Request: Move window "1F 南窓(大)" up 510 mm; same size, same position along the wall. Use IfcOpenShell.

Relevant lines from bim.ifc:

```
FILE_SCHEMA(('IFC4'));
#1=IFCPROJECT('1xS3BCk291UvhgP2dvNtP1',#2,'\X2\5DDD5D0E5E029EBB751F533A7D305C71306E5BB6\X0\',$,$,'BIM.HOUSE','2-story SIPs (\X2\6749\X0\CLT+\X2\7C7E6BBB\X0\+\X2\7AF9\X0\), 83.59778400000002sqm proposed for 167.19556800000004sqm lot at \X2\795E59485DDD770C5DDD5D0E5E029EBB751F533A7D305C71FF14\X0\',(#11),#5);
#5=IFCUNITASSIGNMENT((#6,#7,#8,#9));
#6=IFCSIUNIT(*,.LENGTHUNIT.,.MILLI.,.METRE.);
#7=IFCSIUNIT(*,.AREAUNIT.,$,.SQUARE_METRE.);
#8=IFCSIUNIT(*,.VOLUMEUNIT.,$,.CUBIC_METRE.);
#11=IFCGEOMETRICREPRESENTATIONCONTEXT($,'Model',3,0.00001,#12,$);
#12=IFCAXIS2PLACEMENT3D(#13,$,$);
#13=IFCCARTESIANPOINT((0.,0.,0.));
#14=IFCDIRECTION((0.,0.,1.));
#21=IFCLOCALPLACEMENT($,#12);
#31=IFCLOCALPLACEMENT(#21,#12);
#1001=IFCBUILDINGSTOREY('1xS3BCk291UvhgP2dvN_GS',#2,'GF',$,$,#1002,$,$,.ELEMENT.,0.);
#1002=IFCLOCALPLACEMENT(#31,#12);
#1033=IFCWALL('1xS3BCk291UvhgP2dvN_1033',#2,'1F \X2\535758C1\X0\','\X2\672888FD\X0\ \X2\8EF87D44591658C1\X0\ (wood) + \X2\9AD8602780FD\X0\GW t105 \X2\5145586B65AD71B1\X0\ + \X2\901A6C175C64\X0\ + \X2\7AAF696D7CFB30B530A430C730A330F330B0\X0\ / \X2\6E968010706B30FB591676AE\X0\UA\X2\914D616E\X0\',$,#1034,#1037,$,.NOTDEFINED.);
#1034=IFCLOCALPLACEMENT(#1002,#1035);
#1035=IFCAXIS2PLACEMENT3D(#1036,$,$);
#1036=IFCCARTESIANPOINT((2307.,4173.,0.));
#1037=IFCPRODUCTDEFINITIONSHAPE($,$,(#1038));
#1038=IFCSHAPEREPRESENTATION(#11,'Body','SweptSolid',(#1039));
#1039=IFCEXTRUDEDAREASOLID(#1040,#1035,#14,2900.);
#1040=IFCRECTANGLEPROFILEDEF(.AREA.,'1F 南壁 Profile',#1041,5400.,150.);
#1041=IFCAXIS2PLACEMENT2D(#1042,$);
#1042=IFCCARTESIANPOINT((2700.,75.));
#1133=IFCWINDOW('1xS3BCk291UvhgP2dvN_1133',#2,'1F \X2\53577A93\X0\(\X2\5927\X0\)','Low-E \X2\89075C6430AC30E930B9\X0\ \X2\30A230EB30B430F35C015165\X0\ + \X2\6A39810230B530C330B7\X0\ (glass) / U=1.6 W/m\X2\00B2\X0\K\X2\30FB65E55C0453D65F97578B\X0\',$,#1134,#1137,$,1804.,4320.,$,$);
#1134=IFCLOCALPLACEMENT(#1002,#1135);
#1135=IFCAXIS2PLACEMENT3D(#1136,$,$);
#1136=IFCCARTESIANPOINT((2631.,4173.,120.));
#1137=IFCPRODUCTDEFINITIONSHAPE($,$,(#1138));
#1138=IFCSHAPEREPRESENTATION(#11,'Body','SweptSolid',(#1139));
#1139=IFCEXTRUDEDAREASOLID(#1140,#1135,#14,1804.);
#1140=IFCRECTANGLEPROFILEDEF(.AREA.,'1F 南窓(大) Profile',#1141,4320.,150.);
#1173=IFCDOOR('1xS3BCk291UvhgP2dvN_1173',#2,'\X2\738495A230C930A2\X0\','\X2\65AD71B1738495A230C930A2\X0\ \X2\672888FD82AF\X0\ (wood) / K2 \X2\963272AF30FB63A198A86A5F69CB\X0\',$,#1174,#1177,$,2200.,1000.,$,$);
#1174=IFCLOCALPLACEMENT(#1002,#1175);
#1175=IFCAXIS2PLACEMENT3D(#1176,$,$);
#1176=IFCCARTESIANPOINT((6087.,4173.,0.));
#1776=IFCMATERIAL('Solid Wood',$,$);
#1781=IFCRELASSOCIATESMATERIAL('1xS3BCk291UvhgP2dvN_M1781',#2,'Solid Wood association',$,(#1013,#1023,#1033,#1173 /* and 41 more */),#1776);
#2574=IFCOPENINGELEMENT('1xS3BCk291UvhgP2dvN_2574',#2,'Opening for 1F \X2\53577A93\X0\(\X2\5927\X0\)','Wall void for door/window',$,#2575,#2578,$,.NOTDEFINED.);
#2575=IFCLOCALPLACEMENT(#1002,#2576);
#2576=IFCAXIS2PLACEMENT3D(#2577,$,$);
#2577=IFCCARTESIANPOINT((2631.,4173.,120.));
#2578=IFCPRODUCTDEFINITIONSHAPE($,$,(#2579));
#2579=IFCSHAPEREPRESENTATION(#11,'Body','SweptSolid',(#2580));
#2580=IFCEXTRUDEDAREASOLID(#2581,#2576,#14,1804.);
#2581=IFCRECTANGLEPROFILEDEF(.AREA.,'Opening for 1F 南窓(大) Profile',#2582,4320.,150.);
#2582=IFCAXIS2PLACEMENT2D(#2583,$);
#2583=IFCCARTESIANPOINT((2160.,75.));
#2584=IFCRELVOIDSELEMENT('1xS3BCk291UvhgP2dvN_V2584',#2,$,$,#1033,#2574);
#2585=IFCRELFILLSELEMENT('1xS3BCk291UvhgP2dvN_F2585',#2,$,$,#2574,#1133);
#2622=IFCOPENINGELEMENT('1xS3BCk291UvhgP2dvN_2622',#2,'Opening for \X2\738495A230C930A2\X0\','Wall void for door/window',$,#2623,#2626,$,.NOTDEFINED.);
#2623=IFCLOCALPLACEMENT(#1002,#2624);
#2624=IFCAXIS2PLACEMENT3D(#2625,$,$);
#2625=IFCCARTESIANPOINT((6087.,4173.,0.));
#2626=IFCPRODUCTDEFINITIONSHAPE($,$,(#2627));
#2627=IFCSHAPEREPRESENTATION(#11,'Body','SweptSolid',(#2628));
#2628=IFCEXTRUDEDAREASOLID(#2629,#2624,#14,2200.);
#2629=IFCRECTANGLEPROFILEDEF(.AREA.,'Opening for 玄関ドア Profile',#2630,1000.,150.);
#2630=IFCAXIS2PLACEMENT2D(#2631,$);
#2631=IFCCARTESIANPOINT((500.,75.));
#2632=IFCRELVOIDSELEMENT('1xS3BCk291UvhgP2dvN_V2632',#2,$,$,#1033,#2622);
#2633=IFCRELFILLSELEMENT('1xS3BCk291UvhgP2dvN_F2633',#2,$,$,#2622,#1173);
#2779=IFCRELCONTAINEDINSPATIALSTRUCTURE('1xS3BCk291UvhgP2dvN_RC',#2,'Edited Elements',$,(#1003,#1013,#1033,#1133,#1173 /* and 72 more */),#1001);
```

```python
import numpy as np
import ifcopenshell
import ifcopenshell.api.geometry
import ifcopenshell.util.placement
import ifcopenshell.util.unit

model = ifcopenshell.open("bim.ifc")
unit_scale = ifcopenshell.util.unit.calculate_unit_scale(model)

window = model.by_guid("1xS3BCk291UvhgP2dvN_1133")
opening = window.FillsVoids[0].RelatingOpeningElement
dz = 510.0

shift = np.array([0.0, 0.0, dz])
# The window is not placed relative to its opening, so move both.
for product in (opening, window):
    matrix = ifcopenshell.util.placement.get_local_placement(product.ObjectPlacement)
    matrix[:3, 3] += shift
    ifcopenshell.api.geometry.edit_object_placement(model, product=product, matrix=matrix, is_si=False)

print(f"moved by {dz * unit_scale:+.3f} m")

model.write("bim_rev.ifc")
```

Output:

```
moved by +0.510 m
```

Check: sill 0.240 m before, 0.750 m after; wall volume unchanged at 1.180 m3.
